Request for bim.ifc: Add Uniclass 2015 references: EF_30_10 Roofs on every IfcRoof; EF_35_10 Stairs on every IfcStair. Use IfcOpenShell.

First a look at what the model holds.

```python
import ifcopenshell

model = ifcopenshell.open("bim.ifc")
print(model.schema)
print("classifications:", [c.Name for c in model.by_type("IfcClassification")])
for ifc_class in ("IfcDoor", "IfcRoof", "IfcStair", "IfcWall", "IfcWindow"):
    print(ifc_class, len(model.by_type(ifc_class)))
```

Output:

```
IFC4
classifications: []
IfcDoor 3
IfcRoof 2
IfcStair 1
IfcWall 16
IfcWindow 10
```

```python
import ifcopenshell
import ifcopenshell.api.classification

model = ifcopenshell.open("bim.ifc")

system = ifcopenshell.api.classification.add_classification(model, classification="Uniclass 2015")

codes = {
    "IfcRoof": ("EF_30_10", "Roofs"),
    "IfcStair": ("EF_35_10", "Stairs"),
}
for ifc_class, (code, name) in codes.items():
    products = model.by_type(ifc_class)
    ifcopenshell.api.classification.add_reference(
        model, products=products, classification=system, identification=code, name=name
    )
    print(code, len(products))

model.write("bim_edited.ifc")
```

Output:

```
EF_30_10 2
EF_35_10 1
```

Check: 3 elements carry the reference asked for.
